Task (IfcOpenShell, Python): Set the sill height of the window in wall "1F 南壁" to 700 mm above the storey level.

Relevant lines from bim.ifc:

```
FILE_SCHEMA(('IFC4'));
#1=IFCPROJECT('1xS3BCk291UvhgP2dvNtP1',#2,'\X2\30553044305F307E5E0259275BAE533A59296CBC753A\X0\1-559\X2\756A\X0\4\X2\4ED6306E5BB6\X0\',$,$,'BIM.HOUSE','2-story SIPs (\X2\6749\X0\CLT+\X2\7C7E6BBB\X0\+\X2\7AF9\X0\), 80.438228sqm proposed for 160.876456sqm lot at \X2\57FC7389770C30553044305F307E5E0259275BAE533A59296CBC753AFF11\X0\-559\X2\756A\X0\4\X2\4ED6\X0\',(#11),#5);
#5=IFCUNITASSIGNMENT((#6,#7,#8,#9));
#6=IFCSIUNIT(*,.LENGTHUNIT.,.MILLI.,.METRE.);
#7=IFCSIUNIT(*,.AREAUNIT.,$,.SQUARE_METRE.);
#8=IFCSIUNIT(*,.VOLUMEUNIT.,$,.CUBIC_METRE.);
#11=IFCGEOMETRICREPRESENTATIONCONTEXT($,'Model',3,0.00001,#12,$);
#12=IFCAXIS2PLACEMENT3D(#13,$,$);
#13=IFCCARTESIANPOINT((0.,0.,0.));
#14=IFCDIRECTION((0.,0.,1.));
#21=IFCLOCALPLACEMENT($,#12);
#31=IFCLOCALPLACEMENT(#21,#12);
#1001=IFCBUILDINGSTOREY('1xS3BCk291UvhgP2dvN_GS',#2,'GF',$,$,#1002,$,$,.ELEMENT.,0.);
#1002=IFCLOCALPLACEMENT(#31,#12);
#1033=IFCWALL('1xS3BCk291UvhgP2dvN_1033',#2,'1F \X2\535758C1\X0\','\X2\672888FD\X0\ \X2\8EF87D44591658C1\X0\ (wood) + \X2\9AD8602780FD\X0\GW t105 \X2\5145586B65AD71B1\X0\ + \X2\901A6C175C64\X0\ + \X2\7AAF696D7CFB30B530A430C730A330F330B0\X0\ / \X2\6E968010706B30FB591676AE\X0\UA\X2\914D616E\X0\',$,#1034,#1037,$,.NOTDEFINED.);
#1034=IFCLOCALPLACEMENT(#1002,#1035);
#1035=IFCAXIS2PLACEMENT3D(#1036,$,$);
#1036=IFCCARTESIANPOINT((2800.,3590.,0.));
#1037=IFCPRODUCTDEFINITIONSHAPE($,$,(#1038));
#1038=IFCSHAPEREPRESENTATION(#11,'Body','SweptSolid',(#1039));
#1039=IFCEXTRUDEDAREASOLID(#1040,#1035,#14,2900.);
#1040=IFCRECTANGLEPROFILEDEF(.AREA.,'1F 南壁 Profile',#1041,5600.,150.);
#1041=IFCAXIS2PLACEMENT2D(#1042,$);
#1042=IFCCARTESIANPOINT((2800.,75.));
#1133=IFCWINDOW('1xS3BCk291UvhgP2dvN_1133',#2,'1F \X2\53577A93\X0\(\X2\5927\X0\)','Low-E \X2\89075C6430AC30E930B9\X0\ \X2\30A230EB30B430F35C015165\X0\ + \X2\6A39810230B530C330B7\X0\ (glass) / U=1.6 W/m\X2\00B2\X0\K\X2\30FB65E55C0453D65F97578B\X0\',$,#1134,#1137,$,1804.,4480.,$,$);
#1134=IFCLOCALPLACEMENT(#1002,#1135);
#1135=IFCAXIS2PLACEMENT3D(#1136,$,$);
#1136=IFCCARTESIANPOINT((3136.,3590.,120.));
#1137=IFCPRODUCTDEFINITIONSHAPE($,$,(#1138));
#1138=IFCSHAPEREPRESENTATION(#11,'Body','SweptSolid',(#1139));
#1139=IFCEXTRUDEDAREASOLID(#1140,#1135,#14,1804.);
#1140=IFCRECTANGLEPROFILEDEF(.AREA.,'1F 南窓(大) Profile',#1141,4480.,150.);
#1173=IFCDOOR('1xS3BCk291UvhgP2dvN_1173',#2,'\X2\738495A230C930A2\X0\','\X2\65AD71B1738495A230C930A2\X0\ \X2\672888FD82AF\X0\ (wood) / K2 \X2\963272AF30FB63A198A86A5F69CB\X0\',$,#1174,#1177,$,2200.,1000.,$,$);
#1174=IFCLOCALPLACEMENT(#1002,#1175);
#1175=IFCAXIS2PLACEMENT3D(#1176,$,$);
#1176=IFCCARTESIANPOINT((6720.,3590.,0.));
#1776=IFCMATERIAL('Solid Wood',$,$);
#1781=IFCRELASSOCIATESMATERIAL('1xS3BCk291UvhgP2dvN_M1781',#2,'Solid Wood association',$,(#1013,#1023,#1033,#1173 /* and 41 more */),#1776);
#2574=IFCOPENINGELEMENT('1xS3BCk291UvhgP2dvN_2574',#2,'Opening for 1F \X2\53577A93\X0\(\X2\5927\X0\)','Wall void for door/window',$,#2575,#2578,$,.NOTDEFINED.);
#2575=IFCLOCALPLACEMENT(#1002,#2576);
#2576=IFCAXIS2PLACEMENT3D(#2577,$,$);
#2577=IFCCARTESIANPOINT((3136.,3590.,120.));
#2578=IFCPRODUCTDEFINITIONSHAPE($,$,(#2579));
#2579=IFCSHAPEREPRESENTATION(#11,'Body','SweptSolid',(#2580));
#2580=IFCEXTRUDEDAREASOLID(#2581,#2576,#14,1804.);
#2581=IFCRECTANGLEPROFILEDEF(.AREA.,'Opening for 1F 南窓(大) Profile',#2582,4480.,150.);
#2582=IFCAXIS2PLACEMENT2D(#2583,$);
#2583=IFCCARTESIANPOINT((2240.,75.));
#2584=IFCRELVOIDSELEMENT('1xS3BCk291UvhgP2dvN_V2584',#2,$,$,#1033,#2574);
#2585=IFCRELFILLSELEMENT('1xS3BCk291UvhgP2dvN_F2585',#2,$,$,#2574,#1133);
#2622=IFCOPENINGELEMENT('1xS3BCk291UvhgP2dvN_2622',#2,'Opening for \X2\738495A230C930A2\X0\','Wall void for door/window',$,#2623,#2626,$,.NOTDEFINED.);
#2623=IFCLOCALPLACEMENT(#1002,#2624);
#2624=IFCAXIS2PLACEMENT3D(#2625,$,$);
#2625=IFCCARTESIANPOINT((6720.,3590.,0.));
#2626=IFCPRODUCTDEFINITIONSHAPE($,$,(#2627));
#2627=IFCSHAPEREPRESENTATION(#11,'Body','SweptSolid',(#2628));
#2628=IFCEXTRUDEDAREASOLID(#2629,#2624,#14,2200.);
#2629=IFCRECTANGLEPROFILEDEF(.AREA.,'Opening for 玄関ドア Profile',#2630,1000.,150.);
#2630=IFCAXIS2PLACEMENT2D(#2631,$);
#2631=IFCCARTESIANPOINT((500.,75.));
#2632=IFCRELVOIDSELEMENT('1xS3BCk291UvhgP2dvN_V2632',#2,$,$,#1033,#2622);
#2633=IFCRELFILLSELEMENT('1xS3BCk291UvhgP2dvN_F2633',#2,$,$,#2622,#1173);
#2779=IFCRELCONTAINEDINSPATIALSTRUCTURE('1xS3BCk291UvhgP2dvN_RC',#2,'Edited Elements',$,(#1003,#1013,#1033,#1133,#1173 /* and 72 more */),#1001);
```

```python
import numpy as np
import ifcopenshell
import ifcopenshell.api.geometry
import ifcopenshell.geom
import ifcopenshell.util.element
import ifcopenshell.util.placement
import ifcopenshell.util.shape
import ifcopenshell.util.unit

model = ifcopenshell.open("bim.ifc")
unit_scale = ifcopenshell.util.unit.calculate_unit_scale(model)

window = model.by_id(1133)
opening = window.FillsVoids[0].RelatingOpeningElement
storey = ifcopenshell.util.element.get_container(window, ifc_class="IfcBuildingStorey")
level = ifcopenshell.util.placement.get_local_placement(storey.ObjectPlacement)[2, 3]

# The opening's origin need not be at the sill, so measure its lowest point.
shape = ifcopenshell.geom.create_shape(ifcopenshell.geom.settings(), opening)
bottom = ifcopenshell.util.shape.get_shape_bottom_elevation(shape, shape.geometry) / unit_scale
dz = level + 700.0 - bottom

shift = np.array([0.0, 0.0, dz])
# The window is not placed relative to its opening, so move both.
for product in (opening, window):
    matrix = ifcopenshell.util.placement.get_local_placement(product.ObjectPlacement)
    matrix[:3, 3] += shift
    ifcopenshell.api.geometry.edit_object_placement(model, product=product, matrix=matrix, is_si=False)

print(f"moved by {dz * unit_scale:+.3f} m")

model.write("bim_v2.ifc")
```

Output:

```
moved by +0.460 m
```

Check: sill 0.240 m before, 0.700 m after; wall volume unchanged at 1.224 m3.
